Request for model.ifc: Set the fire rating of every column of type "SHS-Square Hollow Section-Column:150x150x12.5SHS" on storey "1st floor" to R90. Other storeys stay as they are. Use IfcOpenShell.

First a look at what the model holds.

```python
import ifcopenshell
import ifcopenshell.util.element

model = ifcopenshell.open("model.ifc")
print(model.schema)
storey = next(s for s in model.by_type("IfcBuildingStorey") if s.Name == "1st floor")
columns = [e for e in ifcopenshell.util.element.get_decomposition(storey) if e.is_a("IfcColumn")]
seen = {}
for e in columns:
    element_type = ifcopenshell.util.element.get_type(e)
    key = (element_type.Name if element_type != e and element_type else None, ifcopenshell.util.element.get_pset(e, "Pset_ColumnCommon", "FireRating"))
    seen[key] = seen.get(key, 0) + 1
for (name, value), count in sorted(seen.items(), key=str):
    print(count, "x", name, "|", value)
```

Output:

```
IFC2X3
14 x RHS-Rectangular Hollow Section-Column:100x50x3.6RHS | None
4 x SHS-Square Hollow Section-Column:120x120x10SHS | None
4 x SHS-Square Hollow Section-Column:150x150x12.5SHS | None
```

```python
import ifcopenshell
import ifcopenshell.api.pset
import ifcopenshell.util.element

model = ifcopenshell.open("model.ifc")

storey = next(s for s in model.by_type("IfcBuildingStorey") if s.Name == "1st floor")
columns = [e for e in ifcopenshell.util.element.get_decomposition(storey) if e.is_a("IfcColumn")]

count = 0
for e in columns:
    element_type = ifcopenshell.util.element.get_type(e)
    if element_type in (None, e) or element_type.Name != "SHS-Square Hollow Section-Column:150x150x12.5SHS":
        continue
    # add_pset returns the element's existing set when there is one.
    pset = ifcopenshell.api.pset.add_pset(model, product=e, name="Pset_ColumnCommon")
    ifcopenshell.api.pset.edit_pset(model, pset=pset, properties={"FireRating": "R90"})
    count += 1

print(count, "columns updated")

model.write("model-out.ifc")
```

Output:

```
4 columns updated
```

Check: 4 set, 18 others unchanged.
